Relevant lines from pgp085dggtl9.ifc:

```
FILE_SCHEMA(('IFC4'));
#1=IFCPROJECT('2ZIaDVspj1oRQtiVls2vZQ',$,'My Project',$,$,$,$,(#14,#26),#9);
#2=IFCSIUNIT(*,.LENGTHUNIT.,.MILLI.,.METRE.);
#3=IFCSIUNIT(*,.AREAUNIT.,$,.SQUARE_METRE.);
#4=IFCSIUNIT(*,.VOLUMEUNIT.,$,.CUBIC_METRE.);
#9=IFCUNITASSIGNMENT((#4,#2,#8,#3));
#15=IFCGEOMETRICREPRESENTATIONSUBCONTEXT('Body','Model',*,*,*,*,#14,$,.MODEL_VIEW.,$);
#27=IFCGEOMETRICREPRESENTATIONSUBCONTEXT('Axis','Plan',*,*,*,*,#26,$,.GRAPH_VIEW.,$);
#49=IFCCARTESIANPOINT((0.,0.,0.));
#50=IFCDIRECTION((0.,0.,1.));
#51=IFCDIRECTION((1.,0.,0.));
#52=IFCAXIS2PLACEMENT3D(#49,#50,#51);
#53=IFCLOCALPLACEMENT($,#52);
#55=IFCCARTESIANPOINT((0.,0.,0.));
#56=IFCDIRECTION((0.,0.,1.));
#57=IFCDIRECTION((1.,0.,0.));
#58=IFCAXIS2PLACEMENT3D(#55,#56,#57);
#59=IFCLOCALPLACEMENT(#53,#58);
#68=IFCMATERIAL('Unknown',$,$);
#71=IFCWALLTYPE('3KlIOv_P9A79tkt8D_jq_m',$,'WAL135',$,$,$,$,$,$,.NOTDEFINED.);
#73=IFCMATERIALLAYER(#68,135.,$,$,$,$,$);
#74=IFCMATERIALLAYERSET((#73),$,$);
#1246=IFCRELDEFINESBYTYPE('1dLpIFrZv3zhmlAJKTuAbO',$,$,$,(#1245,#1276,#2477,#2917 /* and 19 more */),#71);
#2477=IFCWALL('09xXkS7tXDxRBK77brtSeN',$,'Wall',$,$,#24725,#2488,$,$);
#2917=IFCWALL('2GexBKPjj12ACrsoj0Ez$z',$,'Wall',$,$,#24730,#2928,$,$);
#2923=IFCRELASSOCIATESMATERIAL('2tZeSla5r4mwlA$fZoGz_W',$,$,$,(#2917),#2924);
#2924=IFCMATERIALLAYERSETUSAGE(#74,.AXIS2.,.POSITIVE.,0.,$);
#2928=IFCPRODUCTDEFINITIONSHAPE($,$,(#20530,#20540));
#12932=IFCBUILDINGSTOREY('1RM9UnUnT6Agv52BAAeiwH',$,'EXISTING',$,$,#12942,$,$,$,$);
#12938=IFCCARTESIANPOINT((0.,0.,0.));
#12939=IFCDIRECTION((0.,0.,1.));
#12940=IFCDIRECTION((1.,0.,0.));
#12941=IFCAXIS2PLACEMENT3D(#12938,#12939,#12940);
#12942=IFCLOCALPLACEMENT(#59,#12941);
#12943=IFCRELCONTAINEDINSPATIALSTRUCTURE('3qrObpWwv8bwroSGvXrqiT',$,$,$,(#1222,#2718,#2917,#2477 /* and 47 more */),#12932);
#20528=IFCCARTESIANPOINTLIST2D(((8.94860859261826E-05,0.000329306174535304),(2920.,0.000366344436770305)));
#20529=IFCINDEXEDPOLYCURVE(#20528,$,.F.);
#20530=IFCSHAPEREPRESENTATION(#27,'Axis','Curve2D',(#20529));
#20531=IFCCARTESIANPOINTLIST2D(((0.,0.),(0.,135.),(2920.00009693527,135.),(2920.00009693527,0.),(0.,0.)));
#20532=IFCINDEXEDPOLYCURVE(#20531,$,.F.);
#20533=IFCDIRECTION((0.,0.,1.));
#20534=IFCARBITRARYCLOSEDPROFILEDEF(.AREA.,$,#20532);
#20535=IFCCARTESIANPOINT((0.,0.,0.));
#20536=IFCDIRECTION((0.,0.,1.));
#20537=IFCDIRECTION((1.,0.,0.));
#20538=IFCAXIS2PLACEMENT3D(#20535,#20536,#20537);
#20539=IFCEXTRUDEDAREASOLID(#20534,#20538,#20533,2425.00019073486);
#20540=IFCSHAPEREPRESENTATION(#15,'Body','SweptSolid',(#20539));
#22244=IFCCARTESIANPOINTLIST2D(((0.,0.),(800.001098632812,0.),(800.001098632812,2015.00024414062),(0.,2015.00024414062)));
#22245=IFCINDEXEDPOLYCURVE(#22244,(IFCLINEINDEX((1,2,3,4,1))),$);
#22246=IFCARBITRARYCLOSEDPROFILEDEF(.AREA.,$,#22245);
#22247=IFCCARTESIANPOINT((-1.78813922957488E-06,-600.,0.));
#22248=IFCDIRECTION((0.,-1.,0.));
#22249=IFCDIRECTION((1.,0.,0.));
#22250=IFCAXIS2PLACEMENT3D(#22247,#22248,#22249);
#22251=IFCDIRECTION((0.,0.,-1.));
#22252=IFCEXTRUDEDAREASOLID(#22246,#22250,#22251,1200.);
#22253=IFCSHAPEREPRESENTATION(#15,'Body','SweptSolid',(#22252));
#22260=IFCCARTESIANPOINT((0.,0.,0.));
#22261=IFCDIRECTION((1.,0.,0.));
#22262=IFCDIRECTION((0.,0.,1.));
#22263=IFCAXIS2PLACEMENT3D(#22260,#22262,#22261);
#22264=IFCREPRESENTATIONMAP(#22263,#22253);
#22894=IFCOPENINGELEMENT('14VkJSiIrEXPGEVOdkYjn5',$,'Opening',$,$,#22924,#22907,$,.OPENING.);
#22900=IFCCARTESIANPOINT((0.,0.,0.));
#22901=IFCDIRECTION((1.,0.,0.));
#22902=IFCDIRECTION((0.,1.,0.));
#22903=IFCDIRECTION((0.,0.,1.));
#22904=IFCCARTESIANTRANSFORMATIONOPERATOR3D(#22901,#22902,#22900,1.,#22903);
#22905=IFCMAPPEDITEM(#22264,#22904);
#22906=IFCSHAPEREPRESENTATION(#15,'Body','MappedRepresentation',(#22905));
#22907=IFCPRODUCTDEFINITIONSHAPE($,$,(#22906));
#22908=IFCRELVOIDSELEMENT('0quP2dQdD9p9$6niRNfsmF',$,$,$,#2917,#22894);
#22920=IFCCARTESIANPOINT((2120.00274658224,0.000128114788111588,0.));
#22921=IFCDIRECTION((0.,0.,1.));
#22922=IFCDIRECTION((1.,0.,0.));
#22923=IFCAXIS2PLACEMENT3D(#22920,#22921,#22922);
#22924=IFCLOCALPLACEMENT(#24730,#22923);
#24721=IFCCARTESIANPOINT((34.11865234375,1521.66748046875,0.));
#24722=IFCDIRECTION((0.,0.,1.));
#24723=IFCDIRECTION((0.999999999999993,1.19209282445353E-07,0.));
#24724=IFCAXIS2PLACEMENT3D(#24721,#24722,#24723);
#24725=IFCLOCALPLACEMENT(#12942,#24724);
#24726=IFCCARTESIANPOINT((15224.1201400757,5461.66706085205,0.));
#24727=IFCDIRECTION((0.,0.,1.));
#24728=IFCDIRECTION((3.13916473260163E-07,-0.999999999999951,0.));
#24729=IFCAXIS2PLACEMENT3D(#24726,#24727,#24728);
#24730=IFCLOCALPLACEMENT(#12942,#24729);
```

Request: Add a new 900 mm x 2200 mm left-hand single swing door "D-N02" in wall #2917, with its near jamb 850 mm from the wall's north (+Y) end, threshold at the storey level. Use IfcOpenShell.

```python
import numpy as np
import ifcopenshell
import ifcopenshell.api.feature
import ifcopenshell.api.geometry
import ifcopenshell.api.root
import ifcopenshell.api.spatial
import ifcopenshell.geom
import ifcopenshell.util.element
import ifcopenshell.util.placement
import ifcopenshell.util.representation
import ifcopenshell.util.shape
import ifcopenshell.util.unit

model = ifcopenshell.open("pgp085dggtl9.ifc")
unit_scale = ifcopenshell.util.unit.calculate_unit_scale(model)
settings = ifcopenshell.geom.settings()


def volume(element):
    """Net volume in cubic metres, openings subtracted."""
    shape = ifcopenshell.geom.create_shape(settings, element)
    return ifcopenshell.util.shape.get_volume(shape.geometry)


wall = model.by_guid("2GexBKPjj12ACrsoj0Ez$z")
storey = ifcopenshell.util.element.get_container(wall, ifc_class="IfcBuildingStorey")
context = ifcopenshell.util.representation.get_context(model, "Model", "Body", "MODEL_VIEW")
before = volume(wall)

width, height, from_end, sill = 0.9, 2.2, 0.85, 0.0  # metres

# The wall runs along its own X axis, and the end named is its -X end.
wall_shape = ifcopenshell.geom.create_shape(settings, wall)
x, y, z = ifcopenshell.util.shape.get_vertices(wall_shape.geometry).T
start = x.min() + from_end
face, thickness = float(y.min()), float(y.max() - y.min())
wall_matrix = ifcopenshell.util.placement.get_local_placement(wall.ObjectPlacement)
level = ifcopenshell.util.placement.get_local_placement(storey.ObjectPlacement)[2, 3]


def in_wall(x, y):
    """Placement at x, y metres in the wall's axes, at sill height."""
    matrix = wall_matrix.copy()
    matrix[:, 3] = wall_matrix @ np.array([x / unit_scale, y / unit_scale, 0.0, 1.0])
    matrix[2, 3] = level + sill / unit_scale
    return matrix


# Opening: a box that overshoots both wall faces by 50 mm.
opening = ifcopenshell.api.root.create_entity(model, ifc_class="IfcOpeningElement", predefined_type="OPENING")
box = ifcopenshell.api.geometry.add_wall_representation(
    model, context=context, length=width, height=height, thickness=thickness + 0.1
)
ifcopenshell.api.geometry.assign_representation(model, product=opening, representation=box)
ifcopenshell.api.geometry.edit_object_placement(model, product=opening, matrix=in_wall(start, face - 0.05), is_si=False)
ifcopenshell.api.feature.add_feature(model, feature=opening, element=wall)

door = ifcopenshell.api.root.create_entity(model, ifc_class="IfcDoor", name="D-N02", predefined_type="DOOR")
door.OverallWidth, door.OverallHeight = width / unit_scale, height / unit_scale
door.OperationType = "SINGLE_SWING_LEFT"
body = ifcopenshell.api.geometry.add_door_representation(
    model,
    context=context,
    overall_width=door.OverallWidth,
    overall_height=door.OverallHeight,
    operation_type="SINGLE_SWING_LEFT",
    lining_properties={"LiningDepth": thickness / unit_scale, "ThresholdDepth": thickness / unit_scale},
)
ifcopenshell.api.geometry.assign_representation(model, product=door, representation=body)
ifcopenshell.api.spatial.assign_container(model, products=[door], relating_structure=storey)
ifcopenshell.api.feature.add_filling(model, opening=opening, element=door)

# The lining spans the wall, so the door starts at the wall face.
ifcopenshell.api.geometry.edit_object_placement(model, product=door, matrix=in_wall(start, face), is_si=False)

after = volume(wall)

print(f"wall volume {before:.3f} -> {after:.3f} m3")

model.write("pgp085dggtl9_updated.ifc")
```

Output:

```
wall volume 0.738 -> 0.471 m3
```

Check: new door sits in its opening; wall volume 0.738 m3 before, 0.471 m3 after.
